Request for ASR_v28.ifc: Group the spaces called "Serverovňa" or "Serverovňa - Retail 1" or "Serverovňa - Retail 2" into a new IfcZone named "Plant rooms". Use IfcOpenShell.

First a look at what the model holds.

```python
import ifcopenshell

model = ifcopenshell.open("ASR_v28.ifc")
print(model.schema)
seen = {}
for space in model.by_type("IfcSpace"):
    seen[space.LongName] = seen.get(space.LongName, 0) + 1
for name, count in sorted(seen.items(), key=str):
    print(count, "x", name)
print("zones:", [z.Name for z in model.by_type("IfcZone")][:20])
```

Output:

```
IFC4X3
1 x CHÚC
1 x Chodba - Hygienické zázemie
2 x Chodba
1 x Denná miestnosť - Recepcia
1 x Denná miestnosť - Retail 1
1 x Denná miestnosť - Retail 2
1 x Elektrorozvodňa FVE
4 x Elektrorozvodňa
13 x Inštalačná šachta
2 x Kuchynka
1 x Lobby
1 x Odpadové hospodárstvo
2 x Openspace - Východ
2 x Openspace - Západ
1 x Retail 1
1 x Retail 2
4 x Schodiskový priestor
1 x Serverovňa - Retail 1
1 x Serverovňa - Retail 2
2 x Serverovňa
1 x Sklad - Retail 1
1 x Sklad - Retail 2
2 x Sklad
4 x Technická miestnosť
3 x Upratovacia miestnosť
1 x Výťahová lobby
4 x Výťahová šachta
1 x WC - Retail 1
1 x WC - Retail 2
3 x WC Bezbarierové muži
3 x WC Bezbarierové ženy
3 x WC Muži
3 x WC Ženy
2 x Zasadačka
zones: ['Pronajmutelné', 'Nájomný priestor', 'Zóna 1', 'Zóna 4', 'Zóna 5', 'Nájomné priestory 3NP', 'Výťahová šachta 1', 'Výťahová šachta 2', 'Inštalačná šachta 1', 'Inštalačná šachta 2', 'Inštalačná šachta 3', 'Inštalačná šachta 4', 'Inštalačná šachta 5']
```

```python
import ifcopenshell
import ifcopenshell.api.group
import ifcopenshell.api.root

model = ifcopenshell.open("ASR_v28.ifc")

names = {"Serverovňa", "Serverovňa - Retail 1", "Serverovňa - Retail 2"}
spaces = [s for s in model.by_type("IfcSpace") if s.LongName in names]

zone = ifcopenshell.api.root.create_entity(model, ifc_class="IfcZone", name="Plant rooms")
ifcopenshell.api.group.assign_group(model, products=spaces, group=zone)
print(len(spaces), "spaces in", zone.Name)

model.write("ASR_v28_edited.ifc")
```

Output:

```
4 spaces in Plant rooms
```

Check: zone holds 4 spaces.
